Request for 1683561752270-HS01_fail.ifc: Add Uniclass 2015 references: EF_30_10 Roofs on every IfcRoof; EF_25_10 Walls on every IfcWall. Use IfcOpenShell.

First a look at what the model holds.

```python
import ifcopenshell

model = ifcopenshell.open("1683561752270-HS01_fail.ifc")
print(model.schema)
print("classifications:", [c.Name for c in model.by_type("IfcClassification")])
for ifc_class in ("IfcDoor", "IfcRoof", "IfcStair", "IfcWall", "IfcWindow"):
    print(ifc_class, len(model.by_type(ifc_class)))
```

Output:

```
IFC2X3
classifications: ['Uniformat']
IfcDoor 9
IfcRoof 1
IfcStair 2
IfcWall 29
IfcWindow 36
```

```python
import ifcopenshell
import ifcopenshell.api.classification

model = ifcopenshell.open("1683561752270-HS01_fail.ifc")

# IFC2X3 requires Source and Edition and has no link from the project to the system.
system = model.create_entity("IfcClassification", Source="NBS", Edition="2015", Name="Uniclass 2015")

codes = {
    "IfcRoof": ("EF_30_10", "Roofs"),
    "IfcWall": ("EF_25_10", "Walls"),
}
for ifc_class, (code, name) in codes.items():
    products = model.by_type(ifc_class)
    ifcopenshell.api.classification.add_reference(
        model, products=products, classification=system, identification=code, name=name
    )
    print(code, len(products))

model.write("1683561752270-HS01_fail_updated.ifc")
```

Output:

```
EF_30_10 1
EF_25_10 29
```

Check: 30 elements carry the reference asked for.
